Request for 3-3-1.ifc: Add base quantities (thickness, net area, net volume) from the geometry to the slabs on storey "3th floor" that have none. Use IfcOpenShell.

First a look at what the model holds.

```python
import ifcopenshell
import ifcopenshell.util.element
import ifcopenshell.util.unit

model = ifcopenshell.open("3-3-1.ifc")
print(model.schema)
for unit_type in ("LENGTHUNIT", "AREAUNIT", "VOLUMEUNIT"):
    print(unit_type, ifcopenshell.util.unit.calculate_unit_scale(model, unit_type))
storey = next(s for s in model.by_type("IfcBuildingStorey") if s.Name == "3th floor")
slabs = [e for e in ifcopenshell.util.element.get_decomposition(storey) if e.is_a("IfcSlab")]
for e in sorted(slabs, key=lambda e: e.id()):
    print(e.id(), e.is_a(), e.Name, list(ifcopenshell.util.element.get_psets(e, qtos_only=True)), sep=" | ")
```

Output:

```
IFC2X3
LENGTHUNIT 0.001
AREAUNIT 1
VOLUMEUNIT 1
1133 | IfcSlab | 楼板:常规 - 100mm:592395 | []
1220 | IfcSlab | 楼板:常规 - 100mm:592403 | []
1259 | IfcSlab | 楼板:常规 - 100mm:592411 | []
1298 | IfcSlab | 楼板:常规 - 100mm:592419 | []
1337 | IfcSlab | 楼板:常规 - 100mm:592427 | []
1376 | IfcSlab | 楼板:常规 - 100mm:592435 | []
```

```python
import ifcopenshell
import ifcopenshell.api.pset
import ifcopenshell.geom
import ifcopenshell.util.element
import ifcopenshell.util.shape
import ifcopenshell.util.unit

model = ifcopenshell.open("3-3-1.ifc")
unit_scale = ifcopenshell.util.unit.calculate_unit_scale(model)
area_scale = ifcopenshell.util.unit.calculate_unit_scale(model, "AREAUNIT")
volume_scale = ifcopenshell.util.unit.calculate_unit_scale(model, "VOLUMEUNIT")
settings = ifcopenshell.geom.settings()

storey = next(s for s in model.by_type("IfcBuildingStorey") if s.Name == "3th floor")
slabs = [e for e in ifcopenshell.util.element.get_decomposition(storey) if e.is_a("IfcSlab")]

for e in sorted(slabs, key=lambda e: e.id()):
    if ifcopenshell.util.element.get_psets(e, qtos_only=True, should_inherit=False):
        continue
    # Geometry comes back in metres, in the element's own axes.
    shape = ifcopenshell.geom.create_shape(settings, e)
    values = {
        "Width": ifcopenshell.util.shape.get_z(shape.geometry) / unit_scale,
        "NetArea": ifcopenshell.util.shape.get_footprint_area(shape.geometry) / area_scale,
        "NetVolume": ifcopenshell.util.shape.get_volume(shape.geometry) / volume_scale,
    }
    qto = ifcopenshell.api.pset.add_qto(model, product=e, name="BaseQuantities")
    ifcopenshell.api.pset.edit_qto(model, qto=qto, properties=values)
    print(e.id(), {k: round(v, 3) for k, v in values.items()})

model.write("3-3-1_updated.ifc")
```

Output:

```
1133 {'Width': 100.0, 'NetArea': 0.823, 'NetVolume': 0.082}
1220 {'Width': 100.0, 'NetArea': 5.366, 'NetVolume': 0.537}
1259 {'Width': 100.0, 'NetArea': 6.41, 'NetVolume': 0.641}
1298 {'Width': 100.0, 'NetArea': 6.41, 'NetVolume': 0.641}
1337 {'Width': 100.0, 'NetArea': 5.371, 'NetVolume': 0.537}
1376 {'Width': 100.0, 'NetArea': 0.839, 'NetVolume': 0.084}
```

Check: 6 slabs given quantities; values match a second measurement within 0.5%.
